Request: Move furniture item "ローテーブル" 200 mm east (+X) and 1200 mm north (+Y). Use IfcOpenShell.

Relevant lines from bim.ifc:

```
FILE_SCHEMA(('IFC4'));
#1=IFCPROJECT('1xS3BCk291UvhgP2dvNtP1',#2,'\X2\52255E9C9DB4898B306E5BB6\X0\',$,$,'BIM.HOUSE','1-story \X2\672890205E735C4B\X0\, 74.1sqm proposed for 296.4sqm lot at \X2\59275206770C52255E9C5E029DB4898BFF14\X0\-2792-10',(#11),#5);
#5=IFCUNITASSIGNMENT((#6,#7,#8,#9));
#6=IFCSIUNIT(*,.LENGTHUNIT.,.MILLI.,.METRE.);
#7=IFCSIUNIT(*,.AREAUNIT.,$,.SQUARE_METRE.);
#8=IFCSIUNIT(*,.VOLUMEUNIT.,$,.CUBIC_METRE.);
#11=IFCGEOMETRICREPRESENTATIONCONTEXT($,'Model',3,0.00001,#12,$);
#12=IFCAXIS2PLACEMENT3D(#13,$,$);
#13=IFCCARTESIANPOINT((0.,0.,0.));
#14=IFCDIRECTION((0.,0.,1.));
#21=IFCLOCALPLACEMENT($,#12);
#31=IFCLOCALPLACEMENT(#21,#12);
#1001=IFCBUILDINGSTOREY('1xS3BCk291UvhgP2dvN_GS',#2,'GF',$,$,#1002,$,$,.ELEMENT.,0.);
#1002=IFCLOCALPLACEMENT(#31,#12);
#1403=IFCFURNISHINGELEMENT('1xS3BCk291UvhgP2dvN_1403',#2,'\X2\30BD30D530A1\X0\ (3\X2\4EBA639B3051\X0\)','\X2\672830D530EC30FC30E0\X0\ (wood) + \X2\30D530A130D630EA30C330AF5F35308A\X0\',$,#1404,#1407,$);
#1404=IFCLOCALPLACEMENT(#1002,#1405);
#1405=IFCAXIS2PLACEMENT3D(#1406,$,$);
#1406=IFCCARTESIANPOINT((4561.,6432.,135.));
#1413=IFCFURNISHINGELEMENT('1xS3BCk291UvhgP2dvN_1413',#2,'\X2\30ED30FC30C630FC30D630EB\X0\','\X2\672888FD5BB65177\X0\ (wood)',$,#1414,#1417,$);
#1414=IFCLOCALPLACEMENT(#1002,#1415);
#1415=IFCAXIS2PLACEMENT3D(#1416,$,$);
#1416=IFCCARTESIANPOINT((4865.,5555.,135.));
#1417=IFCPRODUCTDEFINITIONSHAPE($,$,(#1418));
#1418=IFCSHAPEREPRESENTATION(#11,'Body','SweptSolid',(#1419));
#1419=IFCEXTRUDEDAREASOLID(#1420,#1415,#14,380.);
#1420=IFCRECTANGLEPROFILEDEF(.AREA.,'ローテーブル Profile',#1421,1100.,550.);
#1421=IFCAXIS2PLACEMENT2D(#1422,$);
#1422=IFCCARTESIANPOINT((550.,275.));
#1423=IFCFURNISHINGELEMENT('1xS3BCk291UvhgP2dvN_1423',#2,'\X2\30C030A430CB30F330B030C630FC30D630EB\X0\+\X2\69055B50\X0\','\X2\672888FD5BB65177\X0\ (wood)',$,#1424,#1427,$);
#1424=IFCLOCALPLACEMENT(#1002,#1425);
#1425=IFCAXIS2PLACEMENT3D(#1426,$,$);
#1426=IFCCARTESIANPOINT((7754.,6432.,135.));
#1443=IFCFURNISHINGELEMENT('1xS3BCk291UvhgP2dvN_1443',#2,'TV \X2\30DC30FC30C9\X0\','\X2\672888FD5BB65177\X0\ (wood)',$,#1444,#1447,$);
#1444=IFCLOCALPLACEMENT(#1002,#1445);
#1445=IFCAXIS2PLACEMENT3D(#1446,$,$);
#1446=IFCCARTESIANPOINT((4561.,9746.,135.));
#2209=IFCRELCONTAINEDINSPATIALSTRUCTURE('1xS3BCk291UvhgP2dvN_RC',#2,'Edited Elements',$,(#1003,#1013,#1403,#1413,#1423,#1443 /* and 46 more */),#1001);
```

```python
import ifcopenshell
import ifcopenshell.api.geometry
import ifcopenshell.util.placement

model = ifcopenshell.open("bim.ifc")

item = model.by_id(1413)
matrix = ifcopenshell.util.placement.get_local_placement(item.ObjectPlacement)
matrix[0, 3] += 200.0
matrix[1, 3] += 1200.0
ifcopenshell.api.geometry.edit_object_placement(model, product=item, matrix=matrix, is_si=False)

print(ifcopenshell.util.placement.get_local_placement(item.ObjectPlacement).round(3) + 0.0)

model.write("bim_updated.ifc")
```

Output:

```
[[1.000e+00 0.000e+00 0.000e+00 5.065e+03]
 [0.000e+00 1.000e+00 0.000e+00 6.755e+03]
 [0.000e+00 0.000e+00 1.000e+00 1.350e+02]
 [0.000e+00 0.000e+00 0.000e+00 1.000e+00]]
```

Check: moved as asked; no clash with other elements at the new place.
